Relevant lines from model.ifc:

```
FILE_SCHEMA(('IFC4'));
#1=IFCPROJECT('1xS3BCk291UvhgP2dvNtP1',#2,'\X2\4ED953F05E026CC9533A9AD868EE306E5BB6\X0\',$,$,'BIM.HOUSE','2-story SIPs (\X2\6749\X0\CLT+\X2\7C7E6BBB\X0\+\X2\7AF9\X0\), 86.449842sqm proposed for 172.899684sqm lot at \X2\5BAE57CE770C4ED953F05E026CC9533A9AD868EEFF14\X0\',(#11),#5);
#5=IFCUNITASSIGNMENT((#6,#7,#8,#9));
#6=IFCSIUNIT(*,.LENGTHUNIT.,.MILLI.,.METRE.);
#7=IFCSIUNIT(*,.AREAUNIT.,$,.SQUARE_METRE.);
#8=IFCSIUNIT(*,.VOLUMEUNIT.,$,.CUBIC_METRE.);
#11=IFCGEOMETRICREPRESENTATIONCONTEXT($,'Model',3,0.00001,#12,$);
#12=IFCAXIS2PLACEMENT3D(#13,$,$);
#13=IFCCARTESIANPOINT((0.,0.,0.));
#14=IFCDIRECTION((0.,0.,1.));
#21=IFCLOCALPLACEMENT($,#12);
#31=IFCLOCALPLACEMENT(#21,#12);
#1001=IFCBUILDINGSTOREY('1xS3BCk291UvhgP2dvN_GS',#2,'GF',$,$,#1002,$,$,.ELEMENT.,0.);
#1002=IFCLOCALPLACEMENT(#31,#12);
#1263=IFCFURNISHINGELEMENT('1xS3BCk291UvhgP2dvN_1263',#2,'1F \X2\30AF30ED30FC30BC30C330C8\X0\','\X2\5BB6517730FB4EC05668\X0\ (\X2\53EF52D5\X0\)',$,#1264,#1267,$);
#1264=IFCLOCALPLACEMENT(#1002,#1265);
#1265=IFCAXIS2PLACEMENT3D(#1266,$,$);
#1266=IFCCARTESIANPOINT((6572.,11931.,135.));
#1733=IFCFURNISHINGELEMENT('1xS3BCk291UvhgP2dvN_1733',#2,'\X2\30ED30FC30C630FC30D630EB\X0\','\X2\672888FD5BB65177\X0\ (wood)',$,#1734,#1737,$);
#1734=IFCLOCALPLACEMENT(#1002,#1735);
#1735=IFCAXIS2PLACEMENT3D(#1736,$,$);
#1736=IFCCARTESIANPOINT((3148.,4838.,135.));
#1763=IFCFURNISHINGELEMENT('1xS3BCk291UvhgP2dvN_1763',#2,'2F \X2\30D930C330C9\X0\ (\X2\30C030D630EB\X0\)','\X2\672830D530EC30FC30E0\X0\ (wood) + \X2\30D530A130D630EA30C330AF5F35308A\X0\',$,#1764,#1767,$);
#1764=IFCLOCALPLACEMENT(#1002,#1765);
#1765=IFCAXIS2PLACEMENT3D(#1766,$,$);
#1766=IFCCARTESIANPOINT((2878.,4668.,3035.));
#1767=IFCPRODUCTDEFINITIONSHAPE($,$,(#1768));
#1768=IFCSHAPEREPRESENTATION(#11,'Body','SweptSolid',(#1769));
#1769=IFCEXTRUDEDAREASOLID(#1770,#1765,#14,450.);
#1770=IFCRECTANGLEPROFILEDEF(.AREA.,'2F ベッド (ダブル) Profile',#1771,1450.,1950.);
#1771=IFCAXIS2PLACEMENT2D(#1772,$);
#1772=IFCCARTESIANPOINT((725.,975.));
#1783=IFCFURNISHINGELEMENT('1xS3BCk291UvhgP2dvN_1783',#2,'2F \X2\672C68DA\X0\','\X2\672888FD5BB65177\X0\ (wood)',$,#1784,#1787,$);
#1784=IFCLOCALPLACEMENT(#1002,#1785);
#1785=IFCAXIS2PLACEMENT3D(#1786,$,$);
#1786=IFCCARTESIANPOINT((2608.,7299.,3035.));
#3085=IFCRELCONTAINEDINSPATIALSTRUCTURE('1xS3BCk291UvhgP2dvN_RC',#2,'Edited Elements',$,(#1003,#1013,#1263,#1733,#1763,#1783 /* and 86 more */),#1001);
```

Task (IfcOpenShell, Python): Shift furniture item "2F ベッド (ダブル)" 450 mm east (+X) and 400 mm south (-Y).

```python
import ifcopenshell
import ifcopenshell.api.geometry
import ifcopenshell.util.placement
import ifcopenshell.util.unit

model = ifcopenshell.open("model.ifc")
unit_scale = ifcopenshell.util.unit.calculate_unit_scale(model)

item = model.by_guid("1xS3BCk291UvhgP2dvN_1763")
matrix = ifcopenshell.util.placement.get_local_placement(item.ObjectPlacement)
matrix[0, 3] += 0.45 / unit_scale
matrix[1, 3] -= 0.4 / unit_scale
ifcopenshell.api.geometry.edit_object_placement(model, product=item, matrix=matrix, is_si=False)

print(ifcopenshell.util.placement.get_local_placement(item.ObjectPlacement).round(3) + 0.0)

model.write("model-out.ifc")
```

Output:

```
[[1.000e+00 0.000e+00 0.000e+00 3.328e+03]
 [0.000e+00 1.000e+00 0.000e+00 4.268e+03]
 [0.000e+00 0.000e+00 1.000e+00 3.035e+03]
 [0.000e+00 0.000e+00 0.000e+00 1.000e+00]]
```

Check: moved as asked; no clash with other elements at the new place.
